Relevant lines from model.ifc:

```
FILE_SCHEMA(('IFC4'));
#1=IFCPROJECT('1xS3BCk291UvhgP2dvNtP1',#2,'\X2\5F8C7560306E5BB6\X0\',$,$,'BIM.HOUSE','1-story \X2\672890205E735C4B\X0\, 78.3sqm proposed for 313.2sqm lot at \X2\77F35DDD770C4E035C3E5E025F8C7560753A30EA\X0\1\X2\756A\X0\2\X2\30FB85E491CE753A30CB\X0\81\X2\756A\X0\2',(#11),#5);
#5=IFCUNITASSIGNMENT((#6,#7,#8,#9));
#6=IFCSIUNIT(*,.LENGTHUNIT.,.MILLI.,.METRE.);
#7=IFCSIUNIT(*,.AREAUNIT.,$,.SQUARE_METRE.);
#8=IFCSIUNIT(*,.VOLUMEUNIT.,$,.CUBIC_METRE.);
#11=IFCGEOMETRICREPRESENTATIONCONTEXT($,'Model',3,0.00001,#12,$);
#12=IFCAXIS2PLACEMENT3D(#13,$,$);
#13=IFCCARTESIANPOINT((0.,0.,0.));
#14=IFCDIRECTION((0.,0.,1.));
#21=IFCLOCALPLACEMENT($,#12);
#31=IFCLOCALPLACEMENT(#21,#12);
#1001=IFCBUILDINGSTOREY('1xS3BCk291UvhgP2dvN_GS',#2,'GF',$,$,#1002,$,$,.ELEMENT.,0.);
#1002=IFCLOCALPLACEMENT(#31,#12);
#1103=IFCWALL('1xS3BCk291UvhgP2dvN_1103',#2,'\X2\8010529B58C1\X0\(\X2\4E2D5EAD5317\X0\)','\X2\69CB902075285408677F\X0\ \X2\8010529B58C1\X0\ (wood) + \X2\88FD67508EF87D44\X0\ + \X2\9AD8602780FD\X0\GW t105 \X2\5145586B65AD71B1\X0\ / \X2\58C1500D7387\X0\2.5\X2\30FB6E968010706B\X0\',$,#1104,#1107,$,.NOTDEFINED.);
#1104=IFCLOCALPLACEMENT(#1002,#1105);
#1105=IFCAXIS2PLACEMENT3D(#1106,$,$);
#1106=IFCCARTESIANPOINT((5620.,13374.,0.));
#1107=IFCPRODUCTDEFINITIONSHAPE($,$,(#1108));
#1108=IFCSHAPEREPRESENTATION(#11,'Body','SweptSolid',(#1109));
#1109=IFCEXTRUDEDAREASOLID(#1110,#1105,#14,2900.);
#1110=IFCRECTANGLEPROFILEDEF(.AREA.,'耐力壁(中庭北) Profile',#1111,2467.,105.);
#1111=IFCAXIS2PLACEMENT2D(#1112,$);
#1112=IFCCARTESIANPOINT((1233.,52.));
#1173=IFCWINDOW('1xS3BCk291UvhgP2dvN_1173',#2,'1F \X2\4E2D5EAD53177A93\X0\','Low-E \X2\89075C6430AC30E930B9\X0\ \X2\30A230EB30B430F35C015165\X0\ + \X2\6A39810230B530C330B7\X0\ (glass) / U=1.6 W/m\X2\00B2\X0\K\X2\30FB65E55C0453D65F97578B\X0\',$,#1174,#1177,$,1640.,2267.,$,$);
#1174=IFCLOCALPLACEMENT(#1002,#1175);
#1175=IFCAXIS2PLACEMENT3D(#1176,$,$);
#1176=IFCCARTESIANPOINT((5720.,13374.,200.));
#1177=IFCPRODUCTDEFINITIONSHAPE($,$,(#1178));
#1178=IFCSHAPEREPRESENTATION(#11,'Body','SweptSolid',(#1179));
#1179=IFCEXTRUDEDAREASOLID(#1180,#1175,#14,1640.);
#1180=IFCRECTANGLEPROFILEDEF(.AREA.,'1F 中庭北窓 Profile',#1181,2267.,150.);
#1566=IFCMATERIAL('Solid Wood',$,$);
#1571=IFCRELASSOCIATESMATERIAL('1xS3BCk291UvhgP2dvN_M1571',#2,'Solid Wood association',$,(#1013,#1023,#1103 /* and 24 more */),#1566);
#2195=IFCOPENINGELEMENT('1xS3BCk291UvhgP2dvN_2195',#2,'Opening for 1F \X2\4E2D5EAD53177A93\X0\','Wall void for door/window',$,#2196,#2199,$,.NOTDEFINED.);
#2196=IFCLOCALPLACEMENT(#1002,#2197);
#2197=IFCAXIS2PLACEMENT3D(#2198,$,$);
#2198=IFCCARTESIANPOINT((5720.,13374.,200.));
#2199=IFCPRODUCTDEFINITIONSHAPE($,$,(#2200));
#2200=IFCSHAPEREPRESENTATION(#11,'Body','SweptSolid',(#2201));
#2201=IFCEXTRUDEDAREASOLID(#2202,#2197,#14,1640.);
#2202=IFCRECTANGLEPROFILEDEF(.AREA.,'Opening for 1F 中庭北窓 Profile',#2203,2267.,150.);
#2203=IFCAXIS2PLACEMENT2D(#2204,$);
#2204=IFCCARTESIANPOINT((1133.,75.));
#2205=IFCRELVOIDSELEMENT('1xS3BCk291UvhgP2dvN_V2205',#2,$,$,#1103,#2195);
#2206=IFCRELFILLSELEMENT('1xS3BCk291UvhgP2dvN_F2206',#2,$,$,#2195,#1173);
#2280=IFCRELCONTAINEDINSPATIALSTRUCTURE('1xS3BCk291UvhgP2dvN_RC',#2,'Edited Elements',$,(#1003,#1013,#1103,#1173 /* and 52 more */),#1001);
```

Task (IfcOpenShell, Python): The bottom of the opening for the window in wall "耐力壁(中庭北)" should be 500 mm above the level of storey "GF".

```python
import numpy as np
import ifcopenshell
import ifcopenshell.api.geometry
import ifcopenshell.geom
import ifcopenshell.util.element
import ifcopenshell.util.placement
import ifcopenshell.util.shape
import ifcopenshell.util.unit

model = ifcopenshell.open("model.ifc")
unit_scale = ifcopenshell.util.unit.calculate_unit_scale(model)

window = model.by_guid("1xS3BCk291UvhgP2dvN_1173")
opening = window.FillsVoids[0].RelatingOpeningElement
storey = ifcopenshell.util.element.get_container(window, ifc_class="IfcBuildingStorey")
level = ifcopenshell.util.placement.get_local_placement(storey.ObjectPlacement)[2, 3]

# The opening's origin need not be at the sill, so measure its lowest point.
shape = ifcopenshell.geom.create_shape(ifcopenshell.geom.settings(), opening)
bottom = ifcopenshell.util.shape.get_shape_bottom_elevation(shape, shape.geometry) / unit_scale
dz = level + 500.0 - bottom

shift = np.array([0.0, 0.0, dz])
# The window is not placed relative to its opening, so move both.
for product in (opening, window):
    matrix = ifcopenshell.util.placement.get_local_placement(product.ObjectPlacement)
    matrix[:3, 3] += shift
    ifcopenshell.api.geometry.edit_object_placement(model, product=product, matrix=matrix, is_si=False)

print(f"moved by {dz * unit_scale:+.3f} m")

model.write("model_v2.ifc")
```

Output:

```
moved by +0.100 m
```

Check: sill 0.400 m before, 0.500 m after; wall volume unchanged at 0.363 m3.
